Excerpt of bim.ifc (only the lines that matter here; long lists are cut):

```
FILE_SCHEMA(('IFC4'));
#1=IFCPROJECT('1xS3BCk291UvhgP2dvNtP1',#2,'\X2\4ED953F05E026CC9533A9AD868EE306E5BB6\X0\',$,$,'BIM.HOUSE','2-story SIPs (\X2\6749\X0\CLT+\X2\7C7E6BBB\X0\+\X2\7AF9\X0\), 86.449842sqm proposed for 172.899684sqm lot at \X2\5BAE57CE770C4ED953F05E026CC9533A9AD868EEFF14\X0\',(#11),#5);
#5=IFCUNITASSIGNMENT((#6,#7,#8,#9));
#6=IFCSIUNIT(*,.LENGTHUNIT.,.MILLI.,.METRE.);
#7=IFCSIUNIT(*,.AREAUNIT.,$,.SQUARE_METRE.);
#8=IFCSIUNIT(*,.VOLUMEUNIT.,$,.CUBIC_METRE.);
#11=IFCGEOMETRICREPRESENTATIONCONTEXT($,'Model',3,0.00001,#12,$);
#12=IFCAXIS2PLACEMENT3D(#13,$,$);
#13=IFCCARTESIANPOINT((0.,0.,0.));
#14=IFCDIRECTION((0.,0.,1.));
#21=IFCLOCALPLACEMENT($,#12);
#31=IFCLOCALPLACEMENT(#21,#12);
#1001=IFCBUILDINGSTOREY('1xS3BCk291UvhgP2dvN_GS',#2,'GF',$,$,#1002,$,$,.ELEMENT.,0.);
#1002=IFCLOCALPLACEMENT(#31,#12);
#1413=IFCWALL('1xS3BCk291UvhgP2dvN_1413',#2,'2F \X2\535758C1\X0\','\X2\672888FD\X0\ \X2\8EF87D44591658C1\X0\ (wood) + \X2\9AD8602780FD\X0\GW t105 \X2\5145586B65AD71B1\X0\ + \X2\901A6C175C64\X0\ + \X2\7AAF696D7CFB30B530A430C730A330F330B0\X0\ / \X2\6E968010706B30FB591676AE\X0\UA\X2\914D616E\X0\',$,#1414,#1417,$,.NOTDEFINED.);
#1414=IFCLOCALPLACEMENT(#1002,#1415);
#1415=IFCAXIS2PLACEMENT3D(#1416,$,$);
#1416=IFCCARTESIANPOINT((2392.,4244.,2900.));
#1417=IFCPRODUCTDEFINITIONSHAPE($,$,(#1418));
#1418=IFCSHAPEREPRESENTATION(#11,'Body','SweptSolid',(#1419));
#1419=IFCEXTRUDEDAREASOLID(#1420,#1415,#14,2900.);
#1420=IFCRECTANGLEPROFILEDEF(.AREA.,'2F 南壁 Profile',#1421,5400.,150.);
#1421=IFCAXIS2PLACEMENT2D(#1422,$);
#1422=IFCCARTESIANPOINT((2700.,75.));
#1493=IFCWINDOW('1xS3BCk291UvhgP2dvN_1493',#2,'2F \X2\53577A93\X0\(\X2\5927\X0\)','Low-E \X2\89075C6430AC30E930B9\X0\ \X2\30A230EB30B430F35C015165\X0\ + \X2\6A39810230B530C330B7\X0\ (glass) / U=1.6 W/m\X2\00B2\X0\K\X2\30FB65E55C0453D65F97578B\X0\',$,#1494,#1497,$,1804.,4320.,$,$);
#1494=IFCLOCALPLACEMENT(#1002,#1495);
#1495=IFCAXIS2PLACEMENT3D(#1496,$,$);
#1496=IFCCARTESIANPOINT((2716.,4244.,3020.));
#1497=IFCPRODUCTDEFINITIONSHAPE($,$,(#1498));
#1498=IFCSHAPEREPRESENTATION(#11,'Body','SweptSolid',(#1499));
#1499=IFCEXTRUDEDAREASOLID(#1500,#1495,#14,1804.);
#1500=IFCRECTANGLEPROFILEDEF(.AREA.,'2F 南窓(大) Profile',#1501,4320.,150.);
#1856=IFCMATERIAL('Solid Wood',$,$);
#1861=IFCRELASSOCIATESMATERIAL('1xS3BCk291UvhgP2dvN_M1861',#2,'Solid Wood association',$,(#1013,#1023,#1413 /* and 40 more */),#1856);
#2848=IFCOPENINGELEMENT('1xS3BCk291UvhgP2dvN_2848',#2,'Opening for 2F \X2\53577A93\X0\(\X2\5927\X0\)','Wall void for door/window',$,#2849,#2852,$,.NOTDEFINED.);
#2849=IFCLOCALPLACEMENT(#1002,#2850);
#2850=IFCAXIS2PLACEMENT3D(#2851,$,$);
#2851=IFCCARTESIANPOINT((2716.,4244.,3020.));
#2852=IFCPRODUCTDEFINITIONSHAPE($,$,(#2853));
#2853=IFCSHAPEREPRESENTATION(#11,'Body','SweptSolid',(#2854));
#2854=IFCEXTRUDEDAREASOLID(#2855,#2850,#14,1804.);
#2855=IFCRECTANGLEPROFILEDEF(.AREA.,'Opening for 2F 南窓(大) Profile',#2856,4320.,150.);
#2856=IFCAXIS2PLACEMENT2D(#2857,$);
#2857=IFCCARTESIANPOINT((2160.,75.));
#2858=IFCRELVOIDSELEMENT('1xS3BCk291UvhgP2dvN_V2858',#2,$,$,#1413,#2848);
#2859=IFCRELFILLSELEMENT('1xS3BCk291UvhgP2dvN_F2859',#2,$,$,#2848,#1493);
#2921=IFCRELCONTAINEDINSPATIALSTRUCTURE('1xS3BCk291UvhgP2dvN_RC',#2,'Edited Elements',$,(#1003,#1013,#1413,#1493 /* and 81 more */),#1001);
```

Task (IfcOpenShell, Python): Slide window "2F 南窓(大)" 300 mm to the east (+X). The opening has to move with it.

```python
import ifcopenshell
import ifcopenshell.api.geometry
import ifcopenshell.util.placement

model = ifcopenshell.open("bim.ifc")

window = model.by_guid("1xS3BCk291UvhgP2dvN_1493")
opening = window.FillsVoids[0].RelatingOpeningElement
wall = opening.VoidsElements[0].RelatingBuildingElement

wall_matrix = ifcopenshell.util.placement.get_local_placement(wall.ObjectPlacement)
shift = wall_matrix[:3, 0] * 300.0
before = ifcopenshell.util.placement.get_local_placement(window.ObjectPlacement)[:3, 3].copy()

# The window is not placed relative to its opening, so move both.
for product in (opening, window):
    matrix = ifcopenshell.util.placement.get_local_placement(product.ObjectPlacement)
    matrix[:3, 3] += shift
    ifcopenshell.api.geometry.edit_object_placement(model, product=product, matrix=matrix, is_si=False)

after = ifcopenshell.util.placement.get_local_placement(window.ObjectPlacement)[:3, 3]
print("window moved by", (after - before).round(3) + 0.0)

model.write("bim_updated.ifc")
```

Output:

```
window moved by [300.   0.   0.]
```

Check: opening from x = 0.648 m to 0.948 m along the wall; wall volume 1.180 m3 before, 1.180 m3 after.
